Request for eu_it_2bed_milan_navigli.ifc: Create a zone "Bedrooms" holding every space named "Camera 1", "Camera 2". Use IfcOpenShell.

First a look at what the model holds.

```python
import ifcopenshell

model = ifcopenshell.open("eu_it_2bed_milan_navigli.ifc")
print(model.schema)
seen = {}
for space in model.by_type("IfcSpace"):
    seen[space.LongName] = seen.get(space.LongName, 0) + 1
for name, count in sorted(seen.items(), key=str):
    print(count, "x", name)
print("zones:", [z.Name for z in model.by_type("IfcZone")][:20])
```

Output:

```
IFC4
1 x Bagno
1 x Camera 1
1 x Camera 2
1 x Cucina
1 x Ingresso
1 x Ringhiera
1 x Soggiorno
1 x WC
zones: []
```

```python
import ifcopenshell
import ifcopenshell.api.group
import ifcopenshell.api.root

model = ifcopenshell.open("eu_it_2bed_milan_navigli.ifc")

names = {"Camera 1", "Camera 2"}
spaces = [s for s in model.by_type("IfcSpace") if s.LongName in names]

zone = ifcopenshell.api.root.create_entity(model, ifc_class="IfcZone", name="Bedrooms")
ifcopenshell.api.group.assign_group(model, products=spaces, group=zone)
print(len(spaces), "spaces in", zone.Name)

model.write("eu_it_2bed_milan_navigli_updated.ifc")
```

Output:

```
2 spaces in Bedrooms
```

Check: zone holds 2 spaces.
